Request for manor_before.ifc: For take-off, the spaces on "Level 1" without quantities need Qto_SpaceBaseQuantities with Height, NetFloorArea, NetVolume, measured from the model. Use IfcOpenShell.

First a look at what the model holds.

```python
import ifcopenshell
import ifcopenshell.util.element
import ifcopenshell.util.unit

model = ifcopenshell.open("manor_before.ifc")
print(model.schema)
for unit_type in ("LENGTHUNIT", "AREAUNIT", "VOLUMEUNIT"):
    print(unit_type, ifcopenshell.util.unit.calculate_unit_scale(model, unit_type))
storey = next(s for s in model.by_type("IfcBuildingStorey") if s.Name == "Level 1")
spaces = [e for e in ifcopenshell.util.element.get_decomposition(storey) if e.is_a("IfcSpace")]
for e in sorted(spaces, key=lambda e: e.id()):
    print(e.id(), e.is_a(), e.Name, list(ifcopenshell.util.element.get_psets(e, qtos_only=True)), sep=" | ")
```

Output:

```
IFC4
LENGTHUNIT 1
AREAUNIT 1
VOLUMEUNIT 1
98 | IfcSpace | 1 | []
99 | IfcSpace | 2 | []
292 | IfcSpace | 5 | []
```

```python
import ifcopenshell
import ifcopenshell.api.pset
import ifcopenshell.geom
import ifcopenshell.util.element
import ifcopenshell.util.shape
import ifcopenshell.util.unit

model = ifcopenshell.open("manor_before.ifc")
unit_scale = ifcopenshell.util.unit.calculate_unit_scale(model)
area_scale = ifcopenshell.util.unit.calculate_unit_scale(model, "AREAUNIT")
volume_scale = ifcopenshell.util.unit.calculate_unit_scale(model, "VOLUMEUNIT")
settings = ifcopenshell.geom.settings()

storey = next(s for s in model.by_type("IfcBuildingStorey") if s.Name == "Level 1")
spaces = [e for e in ifcopenshell.util.element.get_decomposition(storey) if e.is_a("IfcSpace")]

for e in sorted(spaces, key=lambda e: e.id()):
    if ifcopenshell.util.element.get_psets(e, qtos_only=True, should_inherit=False):
        continue
    # Geometry comes back in metres, in the element's own axes.
    shape = ifcopenshell.geom.create_shape(settings, e)
    values = {
        "Height": ifcopenshell.util.shape.get_z(shape.geometry) / unit_scale,
        "NetFloorArea": ifcopenshell.util.shape.get_footprint_area(shape.geometry) / area_scale,
        "NetVolume": ifcopenshell.util.shape.get_volume(shape.geometry) / volume_scale,
    }
    qto = ifcopenshell.api.pset.add_qto(model, product=e, name="Qto_SpaceBaseQuantities")
    ifcopenshell.api.pset.edit_qto(model, qto=qto, properties=values)
    print(e.id(), {k: round(v, 3) for k, v in values.items()})

model.write("manor_before_edited.ifc")
```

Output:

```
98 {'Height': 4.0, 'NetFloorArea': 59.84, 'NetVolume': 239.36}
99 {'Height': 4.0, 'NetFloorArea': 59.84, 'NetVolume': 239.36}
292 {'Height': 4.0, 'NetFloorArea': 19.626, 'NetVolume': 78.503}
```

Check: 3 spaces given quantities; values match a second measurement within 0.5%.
